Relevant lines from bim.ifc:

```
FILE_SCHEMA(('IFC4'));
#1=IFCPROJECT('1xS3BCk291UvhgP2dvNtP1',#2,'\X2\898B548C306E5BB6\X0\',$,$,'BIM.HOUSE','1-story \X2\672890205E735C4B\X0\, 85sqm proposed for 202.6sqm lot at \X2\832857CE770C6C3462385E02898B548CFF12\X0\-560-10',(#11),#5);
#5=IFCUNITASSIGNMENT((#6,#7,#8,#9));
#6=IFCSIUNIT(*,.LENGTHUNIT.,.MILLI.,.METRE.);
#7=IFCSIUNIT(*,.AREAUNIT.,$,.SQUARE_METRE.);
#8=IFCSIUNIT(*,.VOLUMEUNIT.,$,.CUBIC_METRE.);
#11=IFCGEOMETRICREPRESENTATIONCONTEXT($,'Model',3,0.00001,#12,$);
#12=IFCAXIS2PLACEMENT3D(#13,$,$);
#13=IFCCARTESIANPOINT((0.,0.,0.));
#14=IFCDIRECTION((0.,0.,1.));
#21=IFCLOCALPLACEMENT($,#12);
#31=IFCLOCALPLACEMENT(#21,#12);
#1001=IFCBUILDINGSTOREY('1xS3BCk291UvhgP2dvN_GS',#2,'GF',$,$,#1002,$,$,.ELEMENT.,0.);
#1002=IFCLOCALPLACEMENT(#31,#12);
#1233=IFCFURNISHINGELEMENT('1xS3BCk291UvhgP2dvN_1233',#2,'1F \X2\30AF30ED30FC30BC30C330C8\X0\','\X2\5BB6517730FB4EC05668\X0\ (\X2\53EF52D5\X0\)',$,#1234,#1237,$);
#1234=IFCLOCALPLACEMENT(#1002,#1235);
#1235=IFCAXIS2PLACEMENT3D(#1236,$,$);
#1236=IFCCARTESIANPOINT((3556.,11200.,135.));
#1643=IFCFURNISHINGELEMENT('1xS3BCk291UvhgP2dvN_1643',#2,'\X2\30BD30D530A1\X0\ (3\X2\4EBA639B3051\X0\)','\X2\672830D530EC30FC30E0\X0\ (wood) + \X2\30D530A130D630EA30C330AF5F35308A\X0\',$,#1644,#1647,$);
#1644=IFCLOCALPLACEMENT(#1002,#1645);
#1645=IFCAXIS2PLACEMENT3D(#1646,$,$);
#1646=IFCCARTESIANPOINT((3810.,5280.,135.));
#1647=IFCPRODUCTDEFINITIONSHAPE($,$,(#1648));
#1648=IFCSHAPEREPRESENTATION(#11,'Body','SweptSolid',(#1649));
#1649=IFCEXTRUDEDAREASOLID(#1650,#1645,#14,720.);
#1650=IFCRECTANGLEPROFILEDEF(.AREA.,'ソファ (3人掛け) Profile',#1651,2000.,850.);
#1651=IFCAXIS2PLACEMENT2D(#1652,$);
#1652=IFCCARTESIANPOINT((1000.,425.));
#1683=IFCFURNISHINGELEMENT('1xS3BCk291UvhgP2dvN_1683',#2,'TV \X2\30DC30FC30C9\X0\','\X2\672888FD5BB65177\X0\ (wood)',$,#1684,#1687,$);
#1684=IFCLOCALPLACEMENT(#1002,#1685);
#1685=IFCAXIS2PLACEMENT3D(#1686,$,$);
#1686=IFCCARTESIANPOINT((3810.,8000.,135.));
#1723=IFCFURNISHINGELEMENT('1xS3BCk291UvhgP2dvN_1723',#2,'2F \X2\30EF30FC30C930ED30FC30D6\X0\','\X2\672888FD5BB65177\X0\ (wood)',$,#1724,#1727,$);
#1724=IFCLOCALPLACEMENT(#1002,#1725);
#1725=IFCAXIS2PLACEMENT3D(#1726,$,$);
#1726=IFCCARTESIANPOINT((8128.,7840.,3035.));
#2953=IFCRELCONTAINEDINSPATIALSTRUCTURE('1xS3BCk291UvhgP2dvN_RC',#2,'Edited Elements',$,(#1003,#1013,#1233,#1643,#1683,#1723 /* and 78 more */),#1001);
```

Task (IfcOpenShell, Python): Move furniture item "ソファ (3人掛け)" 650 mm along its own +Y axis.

```python
import ifcopenshell
import ifcopenshell.api.geometry
import ifcopenshell.util.placement
import ifcopenshell.util.unit

model = ifcopenshell.open("bim.ifc")
unit_scale = ifcopenshell.util.unit.calculate_unit_scale(model)

item = model.by_guid("1xS3BCk291UvhgP2dvN_1643")
matrix = ifcopenshell.util.placement.get_local_placement(item.ObjectPlacement)
matrix[:3, 3] += matrix[:3, 1] * 0.65 / unit_scale
ifcopenshell.api.geometry.edit_object_placement(model, product=item, matrix=matrix, is_si=False)

print(ifcopenshell.util.placement.get_local_placement(item.ObjectPlacement).round(3) + 0.0)

model.write("bim_updated.ifc")
```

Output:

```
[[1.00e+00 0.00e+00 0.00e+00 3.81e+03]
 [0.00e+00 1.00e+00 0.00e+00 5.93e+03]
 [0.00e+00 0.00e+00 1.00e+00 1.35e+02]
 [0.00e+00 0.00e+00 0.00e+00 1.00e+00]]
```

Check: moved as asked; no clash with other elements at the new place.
